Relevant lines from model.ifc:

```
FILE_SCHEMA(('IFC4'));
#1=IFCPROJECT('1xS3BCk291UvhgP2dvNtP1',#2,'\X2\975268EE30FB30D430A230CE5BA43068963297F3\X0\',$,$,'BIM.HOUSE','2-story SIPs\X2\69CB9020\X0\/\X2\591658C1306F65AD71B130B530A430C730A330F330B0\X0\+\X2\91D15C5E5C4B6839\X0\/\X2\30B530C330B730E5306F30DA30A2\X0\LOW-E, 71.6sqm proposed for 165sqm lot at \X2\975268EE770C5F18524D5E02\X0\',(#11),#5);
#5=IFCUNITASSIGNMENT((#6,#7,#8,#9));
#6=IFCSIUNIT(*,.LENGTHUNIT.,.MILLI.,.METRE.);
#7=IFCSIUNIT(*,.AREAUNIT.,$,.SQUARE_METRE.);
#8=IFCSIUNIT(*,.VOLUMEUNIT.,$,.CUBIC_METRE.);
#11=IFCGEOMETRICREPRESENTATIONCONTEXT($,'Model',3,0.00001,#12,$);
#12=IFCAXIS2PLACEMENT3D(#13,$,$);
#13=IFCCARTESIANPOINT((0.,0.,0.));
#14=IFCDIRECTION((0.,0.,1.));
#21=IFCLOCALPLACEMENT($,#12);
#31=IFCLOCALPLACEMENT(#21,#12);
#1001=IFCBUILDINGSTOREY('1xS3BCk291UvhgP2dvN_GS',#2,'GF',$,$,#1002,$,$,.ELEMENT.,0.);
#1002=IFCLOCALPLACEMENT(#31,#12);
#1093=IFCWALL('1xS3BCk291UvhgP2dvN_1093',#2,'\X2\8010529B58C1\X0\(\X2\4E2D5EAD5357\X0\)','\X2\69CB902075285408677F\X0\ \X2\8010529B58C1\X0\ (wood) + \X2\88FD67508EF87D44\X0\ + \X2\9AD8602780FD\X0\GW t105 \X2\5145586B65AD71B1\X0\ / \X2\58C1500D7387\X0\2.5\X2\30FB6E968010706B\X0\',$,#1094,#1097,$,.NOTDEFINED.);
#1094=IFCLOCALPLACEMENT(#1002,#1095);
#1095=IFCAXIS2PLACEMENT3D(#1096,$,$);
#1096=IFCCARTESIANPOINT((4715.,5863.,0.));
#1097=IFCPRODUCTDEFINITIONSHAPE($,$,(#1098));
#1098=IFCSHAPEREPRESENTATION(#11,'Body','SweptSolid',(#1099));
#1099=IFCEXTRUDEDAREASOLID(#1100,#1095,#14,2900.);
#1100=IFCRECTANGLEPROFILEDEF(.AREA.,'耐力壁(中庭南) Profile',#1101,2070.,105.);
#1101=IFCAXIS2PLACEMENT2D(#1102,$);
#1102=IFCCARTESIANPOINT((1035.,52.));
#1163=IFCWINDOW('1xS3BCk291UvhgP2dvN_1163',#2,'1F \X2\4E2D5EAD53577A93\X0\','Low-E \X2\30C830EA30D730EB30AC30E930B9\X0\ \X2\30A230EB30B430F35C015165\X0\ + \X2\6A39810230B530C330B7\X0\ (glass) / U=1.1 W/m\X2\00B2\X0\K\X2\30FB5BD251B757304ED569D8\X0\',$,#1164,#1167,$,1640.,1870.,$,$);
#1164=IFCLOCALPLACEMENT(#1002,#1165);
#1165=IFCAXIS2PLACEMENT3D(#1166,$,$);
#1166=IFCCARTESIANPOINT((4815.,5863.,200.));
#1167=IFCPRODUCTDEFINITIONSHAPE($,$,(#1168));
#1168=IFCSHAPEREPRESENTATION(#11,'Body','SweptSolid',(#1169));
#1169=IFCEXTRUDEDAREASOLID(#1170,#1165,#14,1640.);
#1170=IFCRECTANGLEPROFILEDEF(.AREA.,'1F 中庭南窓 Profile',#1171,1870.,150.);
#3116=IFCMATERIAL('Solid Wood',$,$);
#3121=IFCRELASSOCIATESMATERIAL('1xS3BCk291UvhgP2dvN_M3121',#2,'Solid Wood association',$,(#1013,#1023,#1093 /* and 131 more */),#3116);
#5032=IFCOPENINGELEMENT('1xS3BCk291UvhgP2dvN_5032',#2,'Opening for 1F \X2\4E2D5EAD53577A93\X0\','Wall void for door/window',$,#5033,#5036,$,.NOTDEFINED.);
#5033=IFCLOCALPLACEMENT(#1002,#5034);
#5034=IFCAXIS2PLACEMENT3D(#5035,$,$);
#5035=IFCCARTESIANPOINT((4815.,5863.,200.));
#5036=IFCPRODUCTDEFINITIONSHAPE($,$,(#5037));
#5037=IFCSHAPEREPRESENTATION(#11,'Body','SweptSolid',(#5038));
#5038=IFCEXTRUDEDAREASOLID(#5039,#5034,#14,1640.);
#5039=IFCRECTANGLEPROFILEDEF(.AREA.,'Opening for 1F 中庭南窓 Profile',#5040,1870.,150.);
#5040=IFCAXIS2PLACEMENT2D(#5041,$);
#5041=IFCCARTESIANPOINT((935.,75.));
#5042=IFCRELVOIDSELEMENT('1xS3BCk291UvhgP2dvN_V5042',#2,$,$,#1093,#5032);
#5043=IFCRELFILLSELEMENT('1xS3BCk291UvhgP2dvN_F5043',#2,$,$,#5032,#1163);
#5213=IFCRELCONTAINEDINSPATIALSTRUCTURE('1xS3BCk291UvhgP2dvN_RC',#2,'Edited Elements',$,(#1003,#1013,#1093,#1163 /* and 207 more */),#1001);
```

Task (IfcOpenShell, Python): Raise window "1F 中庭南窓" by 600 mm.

```python
import numpy as np
import ifcopenshell
import ifcopenshell.api.geometry
import ifcopenshell.util.placement
import ifcopenshell.util.unit

model = ifcopenshell.open("model.ifc")
unit_scale = ifcopenshell.util.unit.calculate_unit_scale(model)

window = model.by_id(1163)
opening = window.FillsVoids[0].RelatingOpeningElement
dz = 0.6 / unit_scale

shift = np.array([0.0, 0.0, dz])
# The window is not placed relative to its opening, so move both.
for product in (opening, window):
    matrix = ifcopenshell.util.placement.get_local_placement(product.ObjectPlacement)
    matrix[:3, 3] += shift
    ifcopenshell.api.geometry.edit_object_placement(model, product=product, matrix=matrix, is_si=False)

print(f"moved by {dz * unit_scale:+.3f} m")

model.write("model-out.ifc")
```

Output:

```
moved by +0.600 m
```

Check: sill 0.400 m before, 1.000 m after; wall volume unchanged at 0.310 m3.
